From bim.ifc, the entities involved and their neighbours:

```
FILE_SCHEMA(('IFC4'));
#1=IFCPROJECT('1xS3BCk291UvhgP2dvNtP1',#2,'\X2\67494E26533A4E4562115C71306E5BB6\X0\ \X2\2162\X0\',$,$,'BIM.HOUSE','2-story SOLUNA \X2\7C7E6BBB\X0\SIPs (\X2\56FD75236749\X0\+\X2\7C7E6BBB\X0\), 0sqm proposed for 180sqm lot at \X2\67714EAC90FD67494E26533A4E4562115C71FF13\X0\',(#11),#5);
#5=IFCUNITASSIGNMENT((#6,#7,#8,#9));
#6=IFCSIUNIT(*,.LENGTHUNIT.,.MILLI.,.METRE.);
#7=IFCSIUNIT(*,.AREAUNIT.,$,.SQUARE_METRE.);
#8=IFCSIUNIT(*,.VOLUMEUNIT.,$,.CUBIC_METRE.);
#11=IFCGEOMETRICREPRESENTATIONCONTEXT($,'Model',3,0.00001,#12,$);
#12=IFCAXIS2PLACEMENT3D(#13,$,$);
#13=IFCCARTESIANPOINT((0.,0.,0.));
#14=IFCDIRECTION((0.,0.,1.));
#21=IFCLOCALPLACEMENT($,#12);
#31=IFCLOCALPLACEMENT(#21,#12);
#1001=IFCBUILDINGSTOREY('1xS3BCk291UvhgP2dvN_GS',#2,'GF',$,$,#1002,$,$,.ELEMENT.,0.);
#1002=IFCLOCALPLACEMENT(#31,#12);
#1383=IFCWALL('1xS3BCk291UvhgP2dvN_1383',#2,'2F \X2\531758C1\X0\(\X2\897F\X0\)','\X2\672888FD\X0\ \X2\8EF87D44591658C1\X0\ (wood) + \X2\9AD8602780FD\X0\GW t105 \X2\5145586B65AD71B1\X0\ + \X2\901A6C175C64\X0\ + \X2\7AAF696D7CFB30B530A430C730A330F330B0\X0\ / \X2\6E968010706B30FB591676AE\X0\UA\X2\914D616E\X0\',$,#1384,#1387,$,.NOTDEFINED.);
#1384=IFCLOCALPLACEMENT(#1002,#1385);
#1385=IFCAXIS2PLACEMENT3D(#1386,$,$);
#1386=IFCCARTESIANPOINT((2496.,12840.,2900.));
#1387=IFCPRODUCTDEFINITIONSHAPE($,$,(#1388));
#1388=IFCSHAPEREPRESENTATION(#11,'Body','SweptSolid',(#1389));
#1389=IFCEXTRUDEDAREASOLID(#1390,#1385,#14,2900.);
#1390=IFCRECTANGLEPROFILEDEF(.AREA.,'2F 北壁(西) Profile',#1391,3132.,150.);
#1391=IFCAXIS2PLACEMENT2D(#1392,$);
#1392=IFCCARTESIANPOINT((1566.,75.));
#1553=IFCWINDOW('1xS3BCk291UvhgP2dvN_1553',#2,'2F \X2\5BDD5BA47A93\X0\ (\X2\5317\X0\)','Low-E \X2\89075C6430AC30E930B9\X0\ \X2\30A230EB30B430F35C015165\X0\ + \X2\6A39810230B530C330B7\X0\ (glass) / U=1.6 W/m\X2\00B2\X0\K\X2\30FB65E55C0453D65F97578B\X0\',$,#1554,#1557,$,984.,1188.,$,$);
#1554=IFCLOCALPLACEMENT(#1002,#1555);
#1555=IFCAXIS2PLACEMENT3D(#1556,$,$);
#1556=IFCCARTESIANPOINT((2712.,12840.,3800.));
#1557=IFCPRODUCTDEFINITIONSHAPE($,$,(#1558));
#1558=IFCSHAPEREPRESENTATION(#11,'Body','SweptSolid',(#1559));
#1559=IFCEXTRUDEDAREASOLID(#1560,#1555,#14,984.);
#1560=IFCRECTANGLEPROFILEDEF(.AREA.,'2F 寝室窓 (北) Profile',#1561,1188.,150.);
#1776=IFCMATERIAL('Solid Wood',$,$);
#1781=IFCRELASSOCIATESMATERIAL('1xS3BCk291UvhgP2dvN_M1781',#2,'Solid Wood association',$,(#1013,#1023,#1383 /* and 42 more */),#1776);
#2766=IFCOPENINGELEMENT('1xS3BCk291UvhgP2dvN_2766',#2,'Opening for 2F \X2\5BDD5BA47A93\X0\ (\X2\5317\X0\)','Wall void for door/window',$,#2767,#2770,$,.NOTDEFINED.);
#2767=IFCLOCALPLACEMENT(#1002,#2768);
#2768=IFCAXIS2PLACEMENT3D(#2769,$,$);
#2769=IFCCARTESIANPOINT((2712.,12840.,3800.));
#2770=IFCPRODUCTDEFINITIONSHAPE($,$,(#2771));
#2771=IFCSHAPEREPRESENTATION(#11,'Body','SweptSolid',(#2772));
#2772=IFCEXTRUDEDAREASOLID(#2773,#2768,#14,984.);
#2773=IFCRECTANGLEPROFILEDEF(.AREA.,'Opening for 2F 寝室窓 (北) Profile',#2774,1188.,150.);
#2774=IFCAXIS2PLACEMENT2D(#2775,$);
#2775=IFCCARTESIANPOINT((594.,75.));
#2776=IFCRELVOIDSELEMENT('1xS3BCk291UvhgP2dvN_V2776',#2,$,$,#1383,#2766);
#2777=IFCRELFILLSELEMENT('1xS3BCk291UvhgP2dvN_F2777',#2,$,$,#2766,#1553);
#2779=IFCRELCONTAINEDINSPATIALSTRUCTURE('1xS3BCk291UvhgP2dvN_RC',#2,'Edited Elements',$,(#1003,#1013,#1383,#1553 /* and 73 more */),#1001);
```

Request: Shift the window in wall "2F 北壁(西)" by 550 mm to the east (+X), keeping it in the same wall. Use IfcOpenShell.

```python
import ifcopenshell
import ifcopenshell.api.geometry
import ifcopenshell.util.placement

model = ifcopenshell.open("bim.ifc")

window = model.by_guid("1xS3BCk291UvhgP2dvN_1553")
opening = window.FillsVoids[0].RelatingOpeningElement
wall = opening.VoidsElements[0].RelatingBuildingElement

wall_matrix = ifcopenshell.util.placement.get_local_placement(wall.ObjectPlacement)
shift = wall_matrix[:3, 0] * 550.0
before = ifcopenshell.util.placement.get_local_placement(window.ObjectPlacement)[:3, 3].copy()

# The window is not placed relative to its opening, so move both.
for product in (opening, window):
    matrix = ifcopenshell.util.placement.get_local_placement(product.ObjectPlacement)
    matrix[:3, 3] += shift
    ifcopenshell.api.geometry.edit_object_placement(model, product=product, matrix=matrix, is_si=False)

after = ifcopenshell.util.placement.get_local_placement(window.ObjectPlacement)[:3, 3]
print("window moved by", (after - before).round(3) + 0.0)

model.write("bim_v2.ifc")
```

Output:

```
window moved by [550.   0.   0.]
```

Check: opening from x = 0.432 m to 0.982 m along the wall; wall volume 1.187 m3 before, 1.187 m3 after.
